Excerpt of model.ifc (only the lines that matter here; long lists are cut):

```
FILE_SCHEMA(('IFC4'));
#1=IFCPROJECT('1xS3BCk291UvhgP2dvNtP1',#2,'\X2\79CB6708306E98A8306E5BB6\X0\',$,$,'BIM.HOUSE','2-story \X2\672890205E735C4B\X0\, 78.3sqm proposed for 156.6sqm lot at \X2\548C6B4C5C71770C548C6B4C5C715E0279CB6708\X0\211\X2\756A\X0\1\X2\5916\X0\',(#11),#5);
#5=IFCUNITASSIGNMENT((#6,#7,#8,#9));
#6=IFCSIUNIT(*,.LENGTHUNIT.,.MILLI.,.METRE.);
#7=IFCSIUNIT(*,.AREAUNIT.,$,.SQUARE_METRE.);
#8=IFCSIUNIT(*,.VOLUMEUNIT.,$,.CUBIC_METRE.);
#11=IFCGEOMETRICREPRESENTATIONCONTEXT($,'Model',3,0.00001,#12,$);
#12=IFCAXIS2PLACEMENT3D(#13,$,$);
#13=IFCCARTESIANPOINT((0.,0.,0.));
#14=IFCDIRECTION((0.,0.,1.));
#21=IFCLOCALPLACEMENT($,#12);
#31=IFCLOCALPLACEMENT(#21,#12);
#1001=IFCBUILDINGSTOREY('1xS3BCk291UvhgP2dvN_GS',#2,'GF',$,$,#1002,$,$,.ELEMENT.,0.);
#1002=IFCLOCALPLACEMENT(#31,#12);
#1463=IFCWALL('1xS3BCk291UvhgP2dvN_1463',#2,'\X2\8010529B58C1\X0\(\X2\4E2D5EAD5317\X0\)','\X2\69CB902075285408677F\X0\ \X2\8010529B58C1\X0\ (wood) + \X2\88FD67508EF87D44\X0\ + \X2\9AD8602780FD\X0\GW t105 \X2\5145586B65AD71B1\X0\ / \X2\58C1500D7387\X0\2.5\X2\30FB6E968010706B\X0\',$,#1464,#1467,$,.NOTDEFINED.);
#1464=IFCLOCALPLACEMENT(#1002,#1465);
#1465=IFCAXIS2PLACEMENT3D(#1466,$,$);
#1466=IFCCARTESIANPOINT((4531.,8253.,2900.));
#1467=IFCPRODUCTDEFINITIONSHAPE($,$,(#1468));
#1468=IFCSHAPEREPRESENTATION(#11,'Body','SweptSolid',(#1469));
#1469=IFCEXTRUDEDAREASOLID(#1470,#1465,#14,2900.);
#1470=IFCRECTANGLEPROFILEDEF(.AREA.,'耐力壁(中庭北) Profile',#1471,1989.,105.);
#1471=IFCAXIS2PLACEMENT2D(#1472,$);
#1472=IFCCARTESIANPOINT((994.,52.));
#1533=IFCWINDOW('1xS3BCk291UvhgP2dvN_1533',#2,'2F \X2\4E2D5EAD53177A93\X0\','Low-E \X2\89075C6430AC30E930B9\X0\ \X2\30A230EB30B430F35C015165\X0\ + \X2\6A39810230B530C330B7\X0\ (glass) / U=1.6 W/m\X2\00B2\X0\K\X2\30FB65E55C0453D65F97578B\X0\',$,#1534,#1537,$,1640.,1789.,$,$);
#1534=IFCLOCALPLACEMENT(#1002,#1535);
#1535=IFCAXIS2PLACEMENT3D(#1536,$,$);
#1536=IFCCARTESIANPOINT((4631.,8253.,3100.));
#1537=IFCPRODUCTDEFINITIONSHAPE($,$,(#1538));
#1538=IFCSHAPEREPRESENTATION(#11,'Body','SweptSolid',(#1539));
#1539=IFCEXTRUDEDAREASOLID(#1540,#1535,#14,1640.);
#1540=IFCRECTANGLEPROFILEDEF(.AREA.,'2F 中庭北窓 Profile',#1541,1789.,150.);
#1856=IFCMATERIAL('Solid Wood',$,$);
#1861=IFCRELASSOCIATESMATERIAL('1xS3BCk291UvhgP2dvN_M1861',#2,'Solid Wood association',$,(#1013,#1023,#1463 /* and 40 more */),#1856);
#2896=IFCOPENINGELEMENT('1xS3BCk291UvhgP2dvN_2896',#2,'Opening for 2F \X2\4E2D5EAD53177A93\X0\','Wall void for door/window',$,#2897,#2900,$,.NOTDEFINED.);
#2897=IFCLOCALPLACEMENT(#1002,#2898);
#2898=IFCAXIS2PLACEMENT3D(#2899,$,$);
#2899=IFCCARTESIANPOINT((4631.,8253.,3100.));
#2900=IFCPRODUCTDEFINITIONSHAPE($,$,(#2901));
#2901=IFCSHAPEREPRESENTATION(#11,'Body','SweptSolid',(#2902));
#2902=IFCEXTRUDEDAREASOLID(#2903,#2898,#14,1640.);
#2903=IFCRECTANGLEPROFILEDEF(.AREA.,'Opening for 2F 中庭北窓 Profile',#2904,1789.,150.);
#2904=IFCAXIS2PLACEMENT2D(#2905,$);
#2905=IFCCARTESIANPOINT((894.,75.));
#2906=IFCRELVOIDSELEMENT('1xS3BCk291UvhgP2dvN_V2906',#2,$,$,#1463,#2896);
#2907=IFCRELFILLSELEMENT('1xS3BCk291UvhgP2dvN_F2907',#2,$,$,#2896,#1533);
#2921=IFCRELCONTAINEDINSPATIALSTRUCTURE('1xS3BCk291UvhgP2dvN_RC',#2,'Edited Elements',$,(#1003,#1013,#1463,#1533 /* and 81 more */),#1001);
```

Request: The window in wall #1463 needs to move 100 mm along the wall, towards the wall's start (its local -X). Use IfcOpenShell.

```python
import ifcopenshell
import ifcopenshell.api.geometry
import ifcopenshell.util.placement

model = ifcopenshell.open("model.ifc")

window = model.by_id(1533)
opening = window.FillsVoids[0].RelatingOpeningElement
wall = opening.VoidsElements[0].RelatingBuildingElement

wall_matrix = ifcopenshell.util.placement.get_local_placement(wall.ObjectPlacement)
shift = wall_matrix[:3, 0] * -100.0
before = ifcopenshell.util.placement.get_local_placement(window.ObjectPlacement)[:3, 3].copy()

# The window is not placed relative to its opening, so move both.
for product in (opening, window):
    matrix = ifcopenshell.util.placement.get_local_placement(product.ObjectPlacement)
    matrix[:3, 3] += shift
    ifcopenshell.api.geometry.edit_object_placement(model, product=product, matrix=matrix, is_si=False)

after = ifcopenshell.util.placement.get_local_placement(window.ObjectPlacement)[:3, 3]
print("window moved by", (after - before).round(3) + 0.0)

model.write("model_v2.ifc")
```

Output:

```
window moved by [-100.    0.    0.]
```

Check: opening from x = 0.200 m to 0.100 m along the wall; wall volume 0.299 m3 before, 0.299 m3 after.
